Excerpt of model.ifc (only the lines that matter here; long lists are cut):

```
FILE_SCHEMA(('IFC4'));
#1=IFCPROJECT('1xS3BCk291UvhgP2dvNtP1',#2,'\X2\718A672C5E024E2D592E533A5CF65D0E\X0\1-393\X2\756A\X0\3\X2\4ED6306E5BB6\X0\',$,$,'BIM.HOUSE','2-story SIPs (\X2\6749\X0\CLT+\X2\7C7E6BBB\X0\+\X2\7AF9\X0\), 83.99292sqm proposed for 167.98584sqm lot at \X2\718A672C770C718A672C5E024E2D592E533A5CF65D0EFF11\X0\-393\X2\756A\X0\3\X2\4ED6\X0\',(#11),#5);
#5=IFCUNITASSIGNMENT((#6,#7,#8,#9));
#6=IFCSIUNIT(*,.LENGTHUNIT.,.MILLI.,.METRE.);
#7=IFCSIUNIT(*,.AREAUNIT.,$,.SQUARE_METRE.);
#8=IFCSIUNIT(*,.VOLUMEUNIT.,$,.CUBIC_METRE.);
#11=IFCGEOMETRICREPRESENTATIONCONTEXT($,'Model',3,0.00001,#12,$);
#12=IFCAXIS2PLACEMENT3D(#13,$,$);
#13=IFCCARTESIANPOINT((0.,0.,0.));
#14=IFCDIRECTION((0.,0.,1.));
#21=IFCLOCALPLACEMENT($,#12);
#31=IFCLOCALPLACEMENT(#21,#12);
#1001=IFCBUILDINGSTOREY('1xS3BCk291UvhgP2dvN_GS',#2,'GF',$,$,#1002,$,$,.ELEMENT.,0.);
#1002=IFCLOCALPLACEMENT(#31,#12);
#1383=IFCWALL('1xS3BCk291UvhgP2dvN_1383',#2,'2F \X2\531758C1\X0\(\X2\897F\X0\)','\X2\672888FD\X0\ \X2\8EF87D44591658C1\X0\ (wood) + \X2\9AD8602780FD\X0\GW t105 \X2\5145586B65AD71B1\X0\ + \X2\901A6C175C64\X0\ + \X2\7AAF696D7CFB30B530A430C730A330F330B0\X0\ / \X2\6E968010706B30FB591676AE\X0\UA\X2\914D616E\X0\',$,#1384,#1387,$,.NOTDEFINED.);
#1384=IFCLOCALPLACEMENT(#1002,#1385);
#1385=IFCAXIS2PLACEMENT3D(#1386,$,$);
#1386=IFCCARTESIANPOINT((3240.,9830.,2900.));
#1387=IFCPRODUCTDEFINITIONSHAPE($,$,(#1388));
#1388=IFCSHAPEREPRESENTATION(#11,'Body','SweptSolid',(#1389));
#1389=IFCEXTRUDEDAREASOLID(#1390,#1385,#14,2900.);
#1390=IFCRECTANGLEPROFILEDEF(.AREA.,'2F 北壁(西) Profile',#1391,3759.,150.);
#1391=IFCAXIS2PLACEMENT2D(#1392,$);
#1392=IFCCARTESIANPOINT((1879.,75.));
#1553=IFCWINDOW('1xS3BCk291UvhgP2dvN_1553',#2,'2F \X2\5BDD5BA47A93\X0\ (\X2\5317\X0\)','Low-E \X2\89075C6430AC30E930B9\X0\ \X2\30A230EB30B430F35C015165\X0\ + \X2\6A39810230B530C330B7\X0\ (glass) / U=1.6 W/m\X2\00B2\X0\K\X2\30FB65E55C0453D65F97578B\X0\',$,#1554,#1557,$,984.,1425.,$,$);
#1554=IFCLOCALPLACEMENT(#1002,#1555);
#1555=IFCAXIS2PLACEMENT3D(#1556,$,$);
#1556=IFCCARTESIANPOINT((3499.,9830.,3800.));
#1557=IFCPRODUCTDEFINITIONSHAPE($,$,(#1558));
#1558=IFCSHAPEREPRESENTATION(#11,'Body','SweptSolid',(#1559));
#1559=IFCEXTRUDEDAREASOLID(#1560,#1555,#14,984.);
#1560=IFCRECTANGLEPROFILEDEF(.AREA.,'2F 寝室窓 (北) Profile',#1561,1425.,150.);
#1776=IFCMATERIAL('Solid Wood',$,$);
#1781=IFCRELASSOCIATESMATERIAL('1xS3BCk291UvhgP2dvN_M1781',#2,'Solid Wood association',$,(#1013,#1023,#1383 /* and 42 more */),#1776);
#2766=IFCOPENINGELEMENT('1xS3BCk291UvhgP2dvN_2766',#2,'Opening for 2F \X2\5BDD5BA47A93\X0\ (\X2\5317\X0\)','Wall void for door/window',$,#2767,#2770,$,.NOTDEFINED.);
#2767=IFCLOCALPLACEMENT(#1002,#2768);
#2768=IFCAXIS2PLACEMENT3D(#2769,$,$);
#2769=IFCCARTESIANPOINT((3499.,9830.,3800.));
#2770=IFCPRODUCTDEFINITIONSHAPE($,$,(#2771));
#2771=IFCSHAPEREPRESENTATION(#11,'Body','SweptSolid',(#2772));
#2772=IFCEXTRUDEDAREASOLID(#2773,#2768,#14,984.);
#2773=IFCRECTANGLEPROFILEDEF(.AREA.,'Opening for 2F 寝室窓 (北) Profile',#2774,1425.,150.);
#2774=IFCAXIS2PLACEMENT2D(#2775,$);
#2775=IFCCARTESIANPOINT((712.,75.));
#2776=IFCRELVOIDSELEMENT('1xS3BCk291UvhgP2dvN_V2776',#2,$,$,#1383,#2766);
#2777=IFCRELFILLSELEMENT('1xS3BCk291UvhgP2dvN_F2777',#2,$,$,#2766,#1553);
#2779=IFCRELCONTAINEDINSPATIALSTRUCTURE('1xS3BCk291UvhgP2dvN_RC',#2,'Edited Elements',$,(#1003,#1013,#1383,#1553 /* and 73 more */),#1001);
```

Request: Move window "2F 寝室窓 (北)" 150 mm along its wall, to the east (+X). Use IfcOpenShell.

```python
import ifcopenshell
import ifcopenshell.api.geometry
import ifcopenshell.util.placement

model = ifcopenshell.open("model.ifc")

window = model.by_guid("1xS3BCk291UvhgP2dvN_1553")
opening = window.FillsVoids[0].RelatingOpeningElement
wall = opening.VoidsElements[0].RelatingBuildingElement

wall_matrix = ifcopenshell.util.placement.get_local_placement(wall.ObjectPlacement)
shift = wall_matrix[:3, 0] * 150.0
before = ifcopenshell.util.placement.get_local_placement(window.ObjectPlacement)[:3, 3].copy()

# The window is not placed relative to its opening, so move both.
for product in (opening, window):
    matrix = ifcopenshell.util.placement.get_local_placement(product.ObjectPlacement)
    matrix[:3, 3] += shift
    ifcopenshell.api.geometry.edit_object_placement(model, product=product, matrix=matrix, is_si=False)

after = ifcopenshell.util.placement.get_local_placement(window.ObjectPlacement)[:3, 3]
print("window moved by", (after - before).round(3) + 0.0)

model.write("model_v2.ifc")
```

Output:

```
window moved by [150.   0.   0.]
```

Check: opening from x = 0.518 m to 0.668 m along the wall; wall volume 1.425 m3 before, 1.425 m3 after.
